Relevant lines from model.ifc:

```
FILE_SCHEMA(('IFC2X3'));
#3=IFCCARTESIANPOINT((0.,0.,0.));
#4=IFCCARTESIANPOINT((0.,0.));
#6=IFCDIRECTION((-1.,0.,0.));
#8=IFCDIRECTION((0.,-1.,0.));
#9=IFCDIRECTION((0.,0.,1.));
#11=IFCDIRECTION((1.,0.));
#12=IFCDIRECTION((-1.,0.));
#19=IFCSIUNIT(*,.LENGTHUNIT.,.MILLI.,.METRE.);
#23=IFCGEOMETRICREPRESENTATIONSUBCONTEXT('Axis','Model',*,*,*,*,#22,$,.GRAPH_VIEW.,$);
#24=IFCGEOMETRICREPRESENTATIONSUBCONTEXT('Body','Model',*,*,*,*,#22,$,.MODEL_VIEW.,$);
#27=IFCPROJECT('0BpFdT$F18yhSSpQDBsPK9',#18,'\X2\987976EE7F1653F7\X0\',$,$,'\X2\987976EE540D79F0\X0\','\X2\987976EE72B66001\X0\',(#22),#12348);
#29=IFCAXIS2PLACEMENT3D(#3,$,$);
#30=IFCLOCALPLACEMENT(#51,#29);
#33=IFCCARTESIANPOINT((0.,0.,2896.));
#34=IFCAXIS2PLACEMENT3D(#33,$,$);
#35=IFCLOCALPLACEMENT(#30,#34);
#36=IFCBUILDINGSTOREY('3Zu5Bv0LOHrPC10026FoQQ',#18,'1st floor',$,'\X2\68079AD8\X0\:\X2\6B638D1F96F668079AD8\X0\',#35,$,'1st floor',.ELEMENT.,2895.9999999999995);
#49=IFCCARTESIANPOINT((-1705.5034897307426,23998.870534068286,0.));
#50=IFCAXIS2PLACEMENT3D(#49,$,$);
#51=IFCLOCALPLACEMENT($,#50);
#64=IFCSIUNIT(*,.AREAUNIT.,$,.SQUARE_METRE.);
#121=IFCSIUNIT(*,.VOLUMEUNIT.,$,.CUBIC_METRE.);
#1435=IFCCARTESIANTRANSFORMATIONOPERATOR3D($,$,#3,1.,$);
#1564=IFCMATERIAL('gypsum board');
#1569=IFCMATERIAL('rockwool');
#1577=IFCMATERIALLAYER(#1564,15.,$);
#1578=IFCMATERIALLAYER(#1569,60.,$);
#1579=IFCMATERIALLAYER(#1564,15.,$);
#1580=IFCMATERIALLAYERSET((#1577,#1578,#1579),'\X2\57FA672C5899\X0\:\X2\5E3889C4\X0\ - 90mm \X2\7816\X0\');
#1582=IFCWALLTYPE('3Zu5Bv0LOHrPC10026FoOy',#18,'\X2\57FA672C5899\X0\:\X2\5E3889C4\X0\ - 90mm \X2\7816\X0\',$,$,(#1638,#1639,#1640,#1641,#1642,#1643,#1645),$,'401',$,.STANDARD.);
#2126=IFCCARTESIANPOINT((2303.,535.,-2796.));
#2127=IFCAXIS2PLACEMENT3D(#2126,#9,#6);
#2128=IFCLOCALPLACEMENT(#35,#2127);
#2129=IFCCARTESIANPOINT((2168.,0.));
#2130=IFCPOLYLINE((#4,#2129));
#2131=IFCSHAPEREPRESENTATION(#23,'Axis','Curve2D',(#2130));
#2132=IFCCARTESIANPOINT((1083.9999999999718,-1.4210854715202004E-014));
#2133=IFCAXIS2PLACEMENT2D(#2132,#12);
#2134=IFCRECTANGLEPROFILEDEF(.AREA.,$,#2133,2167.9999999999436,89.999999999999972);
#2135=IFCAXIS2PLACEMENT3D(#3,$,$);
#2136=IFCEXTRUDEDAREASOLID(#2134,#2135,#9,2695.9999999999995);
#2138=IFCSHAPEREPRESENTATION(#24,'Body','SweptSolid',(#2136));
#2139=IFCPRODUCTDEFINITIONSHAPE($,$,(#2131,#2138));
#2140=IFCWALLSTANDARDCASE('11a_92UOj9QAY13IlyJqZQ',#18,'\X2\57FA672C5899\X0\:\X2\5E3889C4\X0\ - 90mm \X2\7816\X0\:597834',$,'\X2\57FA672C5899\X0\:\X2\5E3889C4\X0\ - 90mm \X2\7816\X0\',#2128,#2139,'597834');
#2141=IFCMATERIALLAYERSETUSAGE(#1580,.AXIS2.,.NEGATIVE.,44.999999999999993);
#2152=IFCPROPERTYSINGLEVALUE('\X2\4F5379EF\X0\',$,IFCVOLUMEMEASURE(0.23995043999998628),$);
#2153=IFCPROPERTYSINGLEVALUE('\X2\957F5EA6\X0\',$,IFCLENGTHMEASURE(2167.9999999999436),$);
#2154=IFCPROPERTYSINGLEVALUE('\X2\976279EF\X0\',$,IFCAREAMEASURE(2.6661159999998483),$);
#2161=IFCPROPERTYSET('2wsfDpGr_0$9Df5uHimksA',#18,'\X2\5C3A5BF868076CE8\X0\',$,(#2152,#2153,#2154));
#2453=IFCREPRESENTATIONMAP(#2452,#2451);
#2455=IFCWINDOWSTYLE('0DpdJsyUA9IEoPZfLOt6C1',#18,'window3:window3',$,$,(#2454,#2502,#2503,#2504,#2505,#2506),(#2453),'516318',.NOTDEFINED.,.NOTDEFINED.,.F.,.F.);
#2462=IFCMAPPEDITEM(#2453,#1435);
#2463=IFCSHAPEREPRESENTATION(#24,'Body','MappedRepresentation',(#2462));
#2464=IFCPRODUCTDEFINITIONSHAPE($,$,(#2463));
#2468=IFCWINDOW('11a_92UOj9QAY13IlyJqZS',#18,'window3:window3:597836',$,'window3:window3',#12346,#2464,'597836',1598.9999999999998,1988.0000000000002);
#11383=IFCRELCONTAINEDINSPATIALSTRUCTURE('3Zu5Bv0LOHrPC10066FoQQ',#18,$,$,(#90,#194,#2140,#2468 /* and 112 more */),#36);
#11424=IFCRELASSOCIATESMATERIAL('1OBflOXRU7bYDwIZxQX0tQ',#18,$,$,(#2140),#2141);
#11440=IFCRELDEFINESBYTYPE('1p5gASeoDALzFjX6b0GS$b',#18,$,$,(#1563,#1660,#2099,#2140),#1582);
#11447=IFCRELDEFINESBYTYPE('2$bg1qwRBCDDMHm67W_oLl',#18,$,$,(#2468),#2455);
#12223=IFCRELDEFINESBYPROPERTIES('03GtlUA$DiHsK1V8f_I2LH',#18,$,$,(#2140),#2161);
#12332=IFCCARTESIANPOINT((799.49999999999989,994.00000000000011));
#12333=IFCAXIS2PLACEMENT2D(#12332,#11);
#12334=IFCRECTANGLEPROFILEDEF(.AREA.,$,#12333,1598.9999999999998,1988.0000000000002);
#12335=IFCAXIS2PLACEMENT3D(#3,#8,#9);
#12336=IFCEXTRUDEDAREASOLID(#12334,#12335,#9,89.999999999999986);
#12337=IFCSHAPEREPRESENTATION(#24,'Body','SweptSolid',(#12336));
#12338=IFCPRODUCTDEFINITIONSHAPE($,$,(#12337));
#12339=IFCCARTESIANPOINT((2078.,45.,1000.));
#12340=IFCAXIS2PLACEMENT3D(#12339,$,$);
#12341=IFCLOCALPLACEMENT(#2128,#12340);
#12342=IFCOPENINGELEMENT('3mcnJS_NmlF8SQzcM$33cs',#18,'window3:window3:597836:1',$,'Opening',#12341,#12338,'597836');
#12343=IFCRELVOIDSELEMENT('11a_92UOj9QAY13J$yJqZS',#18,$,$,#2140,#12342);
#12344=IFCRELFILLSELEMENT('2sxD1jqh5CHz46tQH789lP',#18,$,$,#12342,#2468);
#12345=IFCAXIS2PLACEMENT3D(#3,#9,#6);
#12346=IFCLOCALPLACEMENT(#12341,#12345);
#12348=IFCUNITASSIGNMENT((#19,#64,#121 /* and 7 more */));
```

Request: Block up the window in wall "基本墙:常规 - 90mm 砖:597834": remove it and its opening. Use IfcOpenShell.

```python
import ifcopenshell
import ifcopenshell.api.feature
import ifcopenshell.api.pset
import ifcopenshell.api.root
import ifcopenshell.geom
import ifcopenshell.util.element
import ifcopenshell.util.shape
import ifcopenshell.util.unit

model = ifcopenshell.open("model.ifc")
area_scale = ifcopenshell.util.unit.calculate_unit_scale(model, "AREAUNIT")
volume_scale = ifcopenshell.util.unit.calculate_unit_scale(model, "VOLUMEUNIT")
settings = ifcopenshell.geom.settings()


def volume(element):
    """Net volume in cubic metres, openings subtracted."""
    shape = ifcopenshell.geom.create_shape(settings, element)
    return ifcopenshell.util.shape.get_volume(shape.geometry)


window = model.by_guid("11a_92UOj9QAY13IlyJqZS")
opening = window.FillsVoids[0].RelatingOpeningElement
wall = opening.VoidsElements[0].RelatingBuildingElement
before = volume(wall)

ifcopenshell.api.root.remove_product(model, product=window)
ifcopenshell.api.feature.remove_feature(model, feature=opening)

after = volume(wall)
thickness = 0.09  # wall thickness in metres

# Update the wall's stored quantities.
pset = model.by_id(ifcopenshell.util.element.get_pset(wall, "尺寸标注", should_inherit=False)["id"])
ifcopenshell.api.pset.edit_pset(model, pset=pset, properties={
    "体积": model.create_entity("IfcVolumeMeasure", after / volume_scale),
    "面积": model.create_entity("IfcAreaMeasure", after / thickness / area_scale),
})

print(f"wall volume {before:.3f} -> {after:.3f} m3")

model.write("model-out.ifc")
```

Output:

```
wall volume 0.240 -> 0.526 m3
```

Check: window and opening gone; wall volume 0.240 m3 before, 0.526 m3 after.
